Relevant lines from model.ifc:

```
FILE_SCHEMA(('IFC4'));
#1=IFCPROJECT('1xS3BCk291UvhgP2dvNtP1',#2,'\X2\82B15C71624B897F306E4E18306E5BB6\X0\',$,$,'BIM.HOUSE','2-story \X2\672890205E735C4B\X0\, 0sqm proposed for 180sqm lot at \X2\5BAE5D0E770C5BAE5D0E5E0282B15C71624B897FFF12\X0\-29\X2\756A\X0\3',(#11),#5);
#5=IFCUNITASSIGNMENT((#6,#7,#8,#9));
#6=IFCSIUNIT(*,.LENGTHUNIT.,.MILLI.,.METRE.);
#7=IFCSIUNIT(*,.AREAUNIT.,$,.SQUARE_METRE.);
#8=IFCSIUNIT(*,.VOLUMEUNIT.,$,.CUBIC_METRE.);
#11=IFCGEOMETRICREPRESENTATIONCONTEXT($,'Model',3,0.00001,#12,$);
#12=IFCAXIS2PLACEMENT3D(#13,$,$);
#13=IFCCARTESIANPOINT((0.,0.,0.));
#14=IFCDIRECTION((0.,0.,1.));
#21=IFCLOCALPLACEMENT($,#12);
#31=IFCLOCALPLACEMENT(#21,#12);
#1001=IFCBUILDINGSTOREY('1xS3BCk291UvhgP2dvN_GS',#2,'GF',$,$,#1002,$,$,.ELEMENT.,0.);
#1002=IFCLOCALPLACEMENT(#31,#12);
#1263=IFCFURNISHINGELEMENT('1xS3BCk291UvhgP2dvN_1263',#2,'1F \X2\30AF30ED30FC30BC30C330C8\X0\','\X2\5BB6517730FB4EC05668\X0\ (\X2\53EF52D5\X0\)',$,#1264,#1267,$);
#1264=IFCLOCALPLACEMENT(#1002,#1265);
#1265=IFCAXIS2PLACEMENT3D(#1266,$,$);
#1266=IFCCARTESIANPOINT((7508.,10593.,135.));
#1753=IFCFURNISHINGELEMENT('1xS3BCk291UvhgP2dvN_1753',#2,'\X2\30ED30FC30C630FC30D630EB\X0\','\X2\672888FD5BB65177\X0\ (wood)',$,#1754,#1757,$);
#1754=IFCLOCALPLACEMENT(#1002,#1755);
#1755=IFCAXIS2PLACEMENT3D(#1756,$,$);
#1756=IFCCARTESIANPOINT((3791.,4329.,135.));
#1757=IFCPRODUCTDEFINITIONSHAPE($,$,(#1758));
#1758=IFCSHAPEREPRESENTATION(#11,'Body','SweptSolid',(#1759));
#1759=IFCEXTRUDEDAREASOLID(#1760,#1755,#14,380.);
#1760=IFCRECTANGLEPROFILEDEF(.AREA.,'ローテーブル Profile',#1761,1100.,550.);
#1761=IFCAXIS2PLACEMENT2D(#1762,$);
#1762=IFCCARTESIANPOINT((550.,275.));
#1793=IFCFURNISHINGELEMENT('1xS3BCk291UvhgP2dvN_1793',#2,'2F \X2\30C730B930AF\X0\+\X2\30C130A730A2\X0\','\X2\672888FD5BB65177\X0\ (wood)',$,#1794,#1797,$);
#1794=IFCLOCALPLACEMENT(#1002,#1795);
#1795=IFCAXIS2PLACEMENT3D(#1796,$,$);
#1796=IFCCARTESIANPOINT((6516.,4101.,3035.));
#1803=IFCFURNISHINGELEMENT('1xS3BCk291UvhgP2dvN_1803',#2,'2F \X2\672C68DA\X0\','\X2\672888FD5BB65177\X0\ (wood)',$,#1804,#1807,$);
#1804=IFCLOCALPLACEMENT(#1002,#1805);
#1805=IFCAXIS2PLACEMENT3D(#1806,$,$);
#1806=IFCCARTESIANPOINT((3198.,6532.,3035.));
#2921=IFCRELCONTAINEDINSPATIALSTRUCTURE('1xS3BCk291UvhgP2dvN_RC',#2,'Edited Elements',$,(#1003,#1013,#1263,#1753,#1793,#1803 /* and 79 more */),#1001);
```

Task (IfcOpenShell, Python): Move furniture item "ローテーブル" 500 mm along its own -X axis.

```python
import ifcopenshell
import ifcopenshell.api.geometry
import ifcopenshell.util.placement
import ifcopenshell.util.unit

model = ifcopenshell.open("model.ifc")
unit_scale = ifcopenshell.util.unit.calculate_unit_scale(model)

item = model.by_guid("1xS3BCk291UvhgP2dvN_1753")
matrix = ifcopenshell.util.placement.get_local_placement(item.ObjectPlacement)
matrix[:3, 3] -= matrix[:3, 0] * 0.5 / unit_scale
ifcopenshell.api.geometry.edit_object_placement(model, product=item, matrix=matrix, is_si=False)

print(ifcopenshell.util.placement.get_local_placement(item.ObjectPlacement).round(3) + 0.0)

model.write("model_updated.ifc")
```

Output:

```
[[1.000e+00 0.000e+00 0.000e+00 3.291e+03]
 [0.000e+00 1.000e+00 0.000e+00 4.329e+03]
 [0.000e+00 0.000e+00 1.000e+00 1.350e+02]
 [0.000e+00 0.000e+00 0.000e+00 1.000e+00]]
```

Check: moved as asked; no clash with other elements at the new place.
